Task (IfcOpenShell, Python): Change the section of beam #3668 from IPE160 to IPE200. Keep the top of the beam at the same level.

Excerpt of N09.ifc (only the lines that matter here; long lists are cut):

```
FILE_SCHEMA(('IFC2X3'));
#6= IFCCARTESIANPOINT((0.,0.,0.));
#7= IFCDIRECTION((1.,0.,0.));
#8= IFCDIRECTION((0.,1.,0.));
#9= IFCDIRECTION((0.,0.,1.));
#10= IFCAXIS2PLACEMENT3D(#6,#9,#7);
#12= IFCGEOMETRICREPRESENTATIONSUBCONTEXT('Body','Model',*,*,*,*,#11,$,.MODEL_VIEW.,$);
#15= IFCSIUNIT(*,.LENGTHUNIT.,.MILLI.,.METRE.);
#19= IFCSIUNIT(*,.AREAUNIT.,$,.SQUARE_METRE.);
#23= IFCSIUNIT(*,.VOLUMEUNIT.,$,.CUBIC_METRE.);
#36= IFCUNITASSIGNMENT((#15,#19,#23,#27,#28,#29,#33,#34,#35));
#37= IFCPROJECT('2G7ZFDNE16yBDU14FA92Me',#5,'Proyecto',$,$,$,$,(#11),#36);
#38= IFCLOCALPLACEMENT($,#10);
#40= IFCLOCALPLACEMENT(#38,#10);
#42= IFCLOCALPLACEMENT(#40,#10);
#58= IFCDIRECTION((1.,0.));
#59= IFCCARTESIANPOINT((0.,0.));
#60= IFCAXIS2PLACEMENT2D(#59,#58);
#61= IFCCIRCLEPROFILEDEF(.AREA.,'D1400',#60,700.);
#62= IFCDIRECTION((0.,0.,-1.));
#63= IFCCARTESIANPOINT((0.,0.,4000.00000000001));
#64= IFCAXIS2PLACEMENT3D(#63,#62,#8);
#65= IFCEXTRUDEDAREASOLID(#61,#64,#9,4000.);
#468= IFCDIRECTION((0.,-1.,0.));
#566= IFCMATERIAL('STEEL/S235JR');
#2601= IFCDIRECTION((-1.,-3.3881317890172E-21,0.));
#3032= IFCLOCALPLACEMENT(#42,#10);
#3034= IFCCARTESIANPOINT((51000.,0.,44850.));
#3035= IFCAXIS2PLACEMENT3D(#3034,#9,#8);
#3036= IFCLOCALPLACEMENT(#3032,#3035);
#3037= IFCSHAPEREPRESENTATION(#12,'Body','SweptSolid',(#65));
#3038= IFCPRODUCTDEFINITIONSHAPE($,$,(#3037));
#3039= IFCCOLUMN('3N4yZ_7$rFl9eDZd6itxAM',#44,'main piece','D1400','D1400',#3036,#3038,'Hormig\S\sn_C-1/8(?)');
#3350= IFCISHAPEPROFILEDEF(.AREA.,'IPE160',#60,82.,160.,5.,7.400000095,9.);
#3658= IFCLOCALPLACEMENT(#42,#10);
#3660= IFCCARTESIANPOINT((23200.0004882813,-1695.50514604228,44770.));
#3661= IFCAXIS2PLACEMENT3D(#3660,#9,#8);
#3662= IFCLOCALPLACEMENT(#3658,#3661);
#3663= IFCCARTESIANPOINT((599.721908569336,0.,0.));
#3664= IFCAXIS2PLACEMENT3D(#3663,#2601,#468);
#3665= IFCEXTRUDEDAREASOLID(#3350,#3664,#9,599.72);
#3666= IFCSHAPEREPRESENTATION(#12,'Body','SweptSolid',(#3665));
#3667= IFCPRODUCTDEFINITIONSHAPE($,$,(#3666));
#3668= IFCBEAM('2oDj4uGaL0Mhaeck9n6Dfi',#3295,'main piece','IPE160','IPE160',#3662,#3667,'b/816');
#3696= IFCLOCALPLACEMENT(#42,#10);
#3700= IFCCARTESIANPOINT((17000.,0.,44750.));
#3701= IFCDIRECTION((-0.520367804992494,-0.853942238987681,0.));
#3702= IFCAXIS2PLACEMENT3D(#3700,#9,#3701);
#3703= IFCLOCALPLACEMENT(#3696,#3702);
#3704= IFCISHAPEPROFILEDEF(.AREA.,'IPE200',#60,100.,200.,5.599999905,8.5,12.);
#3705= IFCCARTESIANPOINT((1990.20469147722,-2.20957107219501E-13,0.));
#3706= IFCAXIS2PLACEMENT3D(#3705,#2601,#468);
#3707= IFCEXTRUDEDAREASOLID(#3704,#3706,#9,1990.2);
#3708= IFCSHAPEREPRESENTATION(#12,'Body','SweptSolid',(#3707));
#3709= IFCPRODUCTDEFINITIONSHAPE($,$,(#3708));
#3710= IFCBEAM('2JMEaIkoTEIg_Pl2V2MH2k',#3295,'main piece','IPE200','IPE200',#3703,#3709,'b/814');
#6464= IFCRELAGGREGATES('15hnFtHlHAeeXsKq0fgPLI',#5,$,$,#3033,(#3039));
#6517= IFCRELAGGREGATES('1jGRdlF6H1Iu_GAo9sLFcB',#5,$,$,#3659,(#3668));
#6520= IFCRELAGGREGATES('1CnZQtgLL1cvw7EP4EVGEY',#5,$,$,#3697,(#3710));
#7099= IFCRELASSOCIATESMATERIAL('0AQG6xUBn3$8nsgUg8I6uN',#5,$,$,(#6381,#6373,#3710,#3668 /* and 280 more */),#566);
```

```python
import ifcopenshell
import ifcopenshell.util.element
import ifcopenshell.util.representation

model = ifcopenshell.open("N09.ifc")

member = model.by_id(3668)
source = next(p for p in model.by_type("IfcIShapeProfileDef") if p.ProfileName == "IPE200")

body = ifcopenshell.util.representation.get_representation(member, "Model", "Body")
solid = body.Items[0]
old_profile = solid.SweptArea

# Copy the section's sizes but keep this member's own profile position.
profile = ifcopenshell.util.element.copy(model, source)
# Profiles are centred, so shift by half the change in depth to hold the top.
shift = (old_profile.OverallDepth - profile.OverallDepth) / 2
x, y = old_profile.Position.Location.Coordinates
up = (0.0, 1.0)  # upwards, in the solid's own plane
location = model.createIfcCartesianPoint((x + up[0] * shift, y + up[1] * shift))
profile.Position = model.createIfcAxis2Placement2D(location, old_profile.Position.RefDirection)
solid.SweptArea = profile
if not model.get_total_inverses(old_profile):
    ifcopenshell.util.element.remove_deep2(model, old_profile)
member.Description = member.Description.replace("IPE160", "IPE200")
member.ObjectType = member.ObjectType.replace("IPE160", "IPE200")

print(solid.SweptArea)

model.write("N09_updated.ifc")
```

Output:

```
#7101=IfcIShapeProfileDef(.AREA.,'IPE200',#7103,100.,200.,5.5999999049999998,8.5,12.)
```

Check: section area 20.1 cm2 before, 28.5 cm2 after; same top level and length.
